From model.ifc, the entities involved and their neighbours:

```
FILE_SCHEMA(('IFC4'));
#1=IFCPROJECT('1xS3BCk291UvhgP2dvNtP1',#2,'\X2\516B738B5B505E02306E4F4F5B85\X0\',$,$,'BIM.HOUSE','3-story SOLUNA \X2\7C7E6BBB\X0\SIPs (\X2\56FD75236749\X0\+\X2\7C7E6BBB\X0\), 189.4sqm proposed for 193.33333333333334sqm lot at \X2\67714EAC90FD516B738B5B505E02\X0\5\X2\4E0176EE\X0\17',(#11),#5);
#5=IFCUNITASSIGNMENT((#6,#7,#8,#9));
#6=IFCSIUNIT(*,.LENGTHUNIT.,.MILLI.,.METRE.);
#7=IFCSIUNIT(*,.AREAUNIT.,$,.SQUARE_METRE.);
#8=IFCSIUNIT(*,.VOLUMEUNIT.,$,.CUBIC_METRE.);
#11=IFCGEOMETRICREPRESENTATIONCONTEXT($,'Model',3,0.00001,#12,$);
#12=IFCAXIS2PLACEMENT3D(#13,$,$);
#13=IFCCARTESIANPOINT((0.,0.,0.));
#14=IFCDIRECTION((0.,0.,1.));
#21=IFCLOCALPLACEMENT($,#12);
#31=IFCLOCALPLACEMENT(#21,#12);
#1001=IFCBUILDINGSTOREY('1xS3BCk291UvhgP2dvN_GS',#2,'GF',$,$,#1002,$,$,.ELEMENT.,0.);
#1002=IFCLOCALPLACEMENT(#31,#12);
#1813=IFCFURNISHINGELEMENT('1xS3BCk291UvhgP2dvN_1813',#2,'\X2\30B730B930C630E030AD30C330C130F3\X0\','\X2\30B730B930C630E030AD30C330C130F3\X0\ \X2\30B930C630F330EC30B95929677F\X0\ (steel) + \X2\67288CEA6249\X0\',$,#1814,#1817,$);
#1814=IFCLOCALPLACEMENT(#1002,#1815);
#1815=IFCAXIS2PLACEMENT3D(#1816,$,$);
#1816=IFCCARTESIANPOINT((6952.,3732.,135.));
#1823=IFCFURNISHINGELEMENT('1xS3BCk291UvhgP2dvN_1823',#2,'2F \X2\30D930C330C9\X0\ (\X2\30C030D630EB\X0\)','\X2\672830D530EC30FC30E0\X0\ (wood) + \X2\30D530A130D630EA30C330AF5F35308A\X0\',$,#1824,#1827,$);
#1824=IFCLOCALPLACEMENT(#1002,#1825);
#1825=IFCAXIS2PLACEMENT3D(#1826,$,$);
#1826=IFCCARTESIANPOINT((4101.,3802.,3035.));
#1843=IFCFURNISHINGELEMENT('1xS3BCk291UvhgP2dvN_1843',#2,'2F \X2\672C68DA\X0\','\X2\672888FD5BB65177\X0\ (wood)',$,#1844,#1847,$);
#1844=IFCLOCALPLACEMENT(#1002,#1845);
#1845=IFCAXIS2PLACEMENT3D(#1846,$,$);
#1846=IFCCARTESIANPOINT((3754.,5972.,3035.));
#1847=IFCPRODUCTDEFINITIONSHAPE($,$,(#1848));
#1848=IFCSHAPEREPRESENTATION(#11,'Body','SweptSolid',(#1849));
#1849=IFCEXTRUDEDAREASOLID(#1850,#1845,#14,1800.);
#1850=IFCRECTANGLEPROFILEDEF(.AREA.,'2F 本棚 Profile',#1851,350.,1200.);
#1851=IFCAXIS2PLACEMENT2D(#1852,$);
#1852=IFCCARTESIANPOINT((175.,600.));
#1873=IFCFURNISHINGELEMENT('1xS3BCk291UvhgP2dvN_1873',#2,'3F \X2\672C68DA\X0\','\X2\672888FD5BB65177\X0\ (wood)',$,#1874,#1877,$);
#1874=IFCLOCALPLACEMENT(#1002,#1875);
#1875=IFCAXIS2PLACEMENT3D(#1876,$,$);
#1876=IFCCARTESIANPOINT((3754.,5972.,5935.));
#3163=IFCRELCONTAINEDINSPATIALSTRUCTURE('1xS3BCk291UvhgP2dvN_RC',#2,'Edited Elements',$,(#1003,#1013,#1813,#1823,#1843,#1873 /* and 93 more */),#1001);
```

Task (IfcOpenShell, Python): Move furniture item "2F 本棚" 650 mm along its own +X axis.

```python
import ifcopenshell
import ifcopenshell.api.geometry
import ifcopenshell.util.placement
import ifcopenshell.util.unit

model = ifcopenshell.open("model.ifc")
unit_scale = ifcopenshell.util.unit.calculate_unit_scale(model)

item = model.by_id(1843)
matrix = ifcopenshell.util.placement.get_local_placement(item.ObjectPlacement)
matrix[:3, 3] += matrix[:3, 0] * 0.65 / unit_scale
ifcopenshell.api.geometry.edit_object_placement(model, product=item, matrix=matrix, is_si=False)

print(ifcopenshell.util.placement.get_local_placement(item.ObjectPlacement).round(3) + 0.0)

model.write("model_v2.ifc")
```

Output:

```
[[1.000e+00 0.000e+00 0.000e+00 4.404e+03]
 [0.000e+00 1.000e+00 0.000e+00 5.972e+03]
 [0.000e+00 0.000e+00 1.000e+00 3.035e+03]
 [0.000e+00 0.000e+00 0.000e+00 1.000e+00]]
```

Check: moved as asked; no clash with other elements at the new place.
